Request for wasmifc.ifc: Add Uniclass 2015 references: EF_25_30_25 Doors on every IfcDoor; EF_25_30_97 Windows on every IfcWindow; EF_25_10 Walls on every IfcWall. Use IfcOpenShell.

First a look at what the model holds.

```python
import ifcopenshell

model = ifcopenshell.open("wasmifc.ifc")
print(model.schema)
print("classifications:", [c.Name for c in model.by_type("IfcClassification")])
for ifc_class in ("IfcDoor", "IfcRoof", "IfcStair", "IfcWall", "IfcWindow"):
    print(ifc_class, len(model.by_type(ifc_class)))
```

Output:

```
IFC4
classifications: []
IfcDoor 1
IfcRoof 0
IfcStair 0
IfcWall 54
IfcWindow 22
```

```python
import ifcopenshell
import ifcopenshell.api.classification

model = ifcopenshell.open("wasmifc.ifc")

system = ifcopenshell.api.classification.add_classification(model, classification="Uniclass 2015")

codes = {
    "IfcDoor": ("EF_25_30_25", "Doors"),
    "IfcWindow": ("EF_25_30_97", "Windows"),
    "IfcWall": ("EF_25_10", "Walls"),
}
for ifc_class, (code, name) in codes.items():
    products = model.by_type(ifc_class)
    ifcopenshell.api.classification.add_reference(
        model, products=products, classification=system, identification=code, name=name
    )
    print(code, len(products))

model.write("wasmifc_rev.ifc")
```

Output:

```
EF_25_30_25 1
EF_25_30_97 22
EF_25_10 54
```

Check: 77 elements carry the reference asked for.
